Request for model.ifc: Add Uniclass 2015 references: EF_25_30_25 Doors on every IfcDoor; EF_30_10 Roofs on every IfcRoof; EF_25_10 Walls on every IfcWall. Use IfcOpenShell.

First a look at what the model holds.

```python
import ifcopenshell

model = ifcopenshell.open("model.ifc")
print(model.schema)
print("classifications:", [c.Name for c in model.by_type("IfcClassification")])
for ifc_class in ("IfcDoor", "IfcRoof", "IfcStair", "IfcWall", "IfcWindow"):
    print(ifc_class, len(model.by_type(ifc_class)))
```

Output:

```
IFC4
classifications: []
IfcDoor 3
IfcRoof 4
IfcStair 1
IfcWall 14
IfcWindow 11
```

```python
import ifcopenshell
import ifcopenshell.api.classification

model = ifcopenshell.open("model.ifc")

system = ifcopenshell.api.classification.add_classification(model, classification="Uniclass 2015")

codes = {
    "IfcDoor": ("EF_25_30_25", "Doors"),
    "IfcRoof": ("EF_30_10", "Roofs"),
    "IfcWall": ("EF_25_10", "Walls"),
}
for ifc_class, (code, name) in codes.items():
    products = model.by_type(ifc_class)
    ifcopenshell.api.classification.add_reference(
        model, products=products, classification=system, identification=code, name=name
    )
    print(code, len(products))

model.write("model_v2.ifc")
```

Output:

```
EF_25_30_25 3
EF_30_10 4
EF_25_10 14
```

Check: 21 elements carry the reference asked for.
